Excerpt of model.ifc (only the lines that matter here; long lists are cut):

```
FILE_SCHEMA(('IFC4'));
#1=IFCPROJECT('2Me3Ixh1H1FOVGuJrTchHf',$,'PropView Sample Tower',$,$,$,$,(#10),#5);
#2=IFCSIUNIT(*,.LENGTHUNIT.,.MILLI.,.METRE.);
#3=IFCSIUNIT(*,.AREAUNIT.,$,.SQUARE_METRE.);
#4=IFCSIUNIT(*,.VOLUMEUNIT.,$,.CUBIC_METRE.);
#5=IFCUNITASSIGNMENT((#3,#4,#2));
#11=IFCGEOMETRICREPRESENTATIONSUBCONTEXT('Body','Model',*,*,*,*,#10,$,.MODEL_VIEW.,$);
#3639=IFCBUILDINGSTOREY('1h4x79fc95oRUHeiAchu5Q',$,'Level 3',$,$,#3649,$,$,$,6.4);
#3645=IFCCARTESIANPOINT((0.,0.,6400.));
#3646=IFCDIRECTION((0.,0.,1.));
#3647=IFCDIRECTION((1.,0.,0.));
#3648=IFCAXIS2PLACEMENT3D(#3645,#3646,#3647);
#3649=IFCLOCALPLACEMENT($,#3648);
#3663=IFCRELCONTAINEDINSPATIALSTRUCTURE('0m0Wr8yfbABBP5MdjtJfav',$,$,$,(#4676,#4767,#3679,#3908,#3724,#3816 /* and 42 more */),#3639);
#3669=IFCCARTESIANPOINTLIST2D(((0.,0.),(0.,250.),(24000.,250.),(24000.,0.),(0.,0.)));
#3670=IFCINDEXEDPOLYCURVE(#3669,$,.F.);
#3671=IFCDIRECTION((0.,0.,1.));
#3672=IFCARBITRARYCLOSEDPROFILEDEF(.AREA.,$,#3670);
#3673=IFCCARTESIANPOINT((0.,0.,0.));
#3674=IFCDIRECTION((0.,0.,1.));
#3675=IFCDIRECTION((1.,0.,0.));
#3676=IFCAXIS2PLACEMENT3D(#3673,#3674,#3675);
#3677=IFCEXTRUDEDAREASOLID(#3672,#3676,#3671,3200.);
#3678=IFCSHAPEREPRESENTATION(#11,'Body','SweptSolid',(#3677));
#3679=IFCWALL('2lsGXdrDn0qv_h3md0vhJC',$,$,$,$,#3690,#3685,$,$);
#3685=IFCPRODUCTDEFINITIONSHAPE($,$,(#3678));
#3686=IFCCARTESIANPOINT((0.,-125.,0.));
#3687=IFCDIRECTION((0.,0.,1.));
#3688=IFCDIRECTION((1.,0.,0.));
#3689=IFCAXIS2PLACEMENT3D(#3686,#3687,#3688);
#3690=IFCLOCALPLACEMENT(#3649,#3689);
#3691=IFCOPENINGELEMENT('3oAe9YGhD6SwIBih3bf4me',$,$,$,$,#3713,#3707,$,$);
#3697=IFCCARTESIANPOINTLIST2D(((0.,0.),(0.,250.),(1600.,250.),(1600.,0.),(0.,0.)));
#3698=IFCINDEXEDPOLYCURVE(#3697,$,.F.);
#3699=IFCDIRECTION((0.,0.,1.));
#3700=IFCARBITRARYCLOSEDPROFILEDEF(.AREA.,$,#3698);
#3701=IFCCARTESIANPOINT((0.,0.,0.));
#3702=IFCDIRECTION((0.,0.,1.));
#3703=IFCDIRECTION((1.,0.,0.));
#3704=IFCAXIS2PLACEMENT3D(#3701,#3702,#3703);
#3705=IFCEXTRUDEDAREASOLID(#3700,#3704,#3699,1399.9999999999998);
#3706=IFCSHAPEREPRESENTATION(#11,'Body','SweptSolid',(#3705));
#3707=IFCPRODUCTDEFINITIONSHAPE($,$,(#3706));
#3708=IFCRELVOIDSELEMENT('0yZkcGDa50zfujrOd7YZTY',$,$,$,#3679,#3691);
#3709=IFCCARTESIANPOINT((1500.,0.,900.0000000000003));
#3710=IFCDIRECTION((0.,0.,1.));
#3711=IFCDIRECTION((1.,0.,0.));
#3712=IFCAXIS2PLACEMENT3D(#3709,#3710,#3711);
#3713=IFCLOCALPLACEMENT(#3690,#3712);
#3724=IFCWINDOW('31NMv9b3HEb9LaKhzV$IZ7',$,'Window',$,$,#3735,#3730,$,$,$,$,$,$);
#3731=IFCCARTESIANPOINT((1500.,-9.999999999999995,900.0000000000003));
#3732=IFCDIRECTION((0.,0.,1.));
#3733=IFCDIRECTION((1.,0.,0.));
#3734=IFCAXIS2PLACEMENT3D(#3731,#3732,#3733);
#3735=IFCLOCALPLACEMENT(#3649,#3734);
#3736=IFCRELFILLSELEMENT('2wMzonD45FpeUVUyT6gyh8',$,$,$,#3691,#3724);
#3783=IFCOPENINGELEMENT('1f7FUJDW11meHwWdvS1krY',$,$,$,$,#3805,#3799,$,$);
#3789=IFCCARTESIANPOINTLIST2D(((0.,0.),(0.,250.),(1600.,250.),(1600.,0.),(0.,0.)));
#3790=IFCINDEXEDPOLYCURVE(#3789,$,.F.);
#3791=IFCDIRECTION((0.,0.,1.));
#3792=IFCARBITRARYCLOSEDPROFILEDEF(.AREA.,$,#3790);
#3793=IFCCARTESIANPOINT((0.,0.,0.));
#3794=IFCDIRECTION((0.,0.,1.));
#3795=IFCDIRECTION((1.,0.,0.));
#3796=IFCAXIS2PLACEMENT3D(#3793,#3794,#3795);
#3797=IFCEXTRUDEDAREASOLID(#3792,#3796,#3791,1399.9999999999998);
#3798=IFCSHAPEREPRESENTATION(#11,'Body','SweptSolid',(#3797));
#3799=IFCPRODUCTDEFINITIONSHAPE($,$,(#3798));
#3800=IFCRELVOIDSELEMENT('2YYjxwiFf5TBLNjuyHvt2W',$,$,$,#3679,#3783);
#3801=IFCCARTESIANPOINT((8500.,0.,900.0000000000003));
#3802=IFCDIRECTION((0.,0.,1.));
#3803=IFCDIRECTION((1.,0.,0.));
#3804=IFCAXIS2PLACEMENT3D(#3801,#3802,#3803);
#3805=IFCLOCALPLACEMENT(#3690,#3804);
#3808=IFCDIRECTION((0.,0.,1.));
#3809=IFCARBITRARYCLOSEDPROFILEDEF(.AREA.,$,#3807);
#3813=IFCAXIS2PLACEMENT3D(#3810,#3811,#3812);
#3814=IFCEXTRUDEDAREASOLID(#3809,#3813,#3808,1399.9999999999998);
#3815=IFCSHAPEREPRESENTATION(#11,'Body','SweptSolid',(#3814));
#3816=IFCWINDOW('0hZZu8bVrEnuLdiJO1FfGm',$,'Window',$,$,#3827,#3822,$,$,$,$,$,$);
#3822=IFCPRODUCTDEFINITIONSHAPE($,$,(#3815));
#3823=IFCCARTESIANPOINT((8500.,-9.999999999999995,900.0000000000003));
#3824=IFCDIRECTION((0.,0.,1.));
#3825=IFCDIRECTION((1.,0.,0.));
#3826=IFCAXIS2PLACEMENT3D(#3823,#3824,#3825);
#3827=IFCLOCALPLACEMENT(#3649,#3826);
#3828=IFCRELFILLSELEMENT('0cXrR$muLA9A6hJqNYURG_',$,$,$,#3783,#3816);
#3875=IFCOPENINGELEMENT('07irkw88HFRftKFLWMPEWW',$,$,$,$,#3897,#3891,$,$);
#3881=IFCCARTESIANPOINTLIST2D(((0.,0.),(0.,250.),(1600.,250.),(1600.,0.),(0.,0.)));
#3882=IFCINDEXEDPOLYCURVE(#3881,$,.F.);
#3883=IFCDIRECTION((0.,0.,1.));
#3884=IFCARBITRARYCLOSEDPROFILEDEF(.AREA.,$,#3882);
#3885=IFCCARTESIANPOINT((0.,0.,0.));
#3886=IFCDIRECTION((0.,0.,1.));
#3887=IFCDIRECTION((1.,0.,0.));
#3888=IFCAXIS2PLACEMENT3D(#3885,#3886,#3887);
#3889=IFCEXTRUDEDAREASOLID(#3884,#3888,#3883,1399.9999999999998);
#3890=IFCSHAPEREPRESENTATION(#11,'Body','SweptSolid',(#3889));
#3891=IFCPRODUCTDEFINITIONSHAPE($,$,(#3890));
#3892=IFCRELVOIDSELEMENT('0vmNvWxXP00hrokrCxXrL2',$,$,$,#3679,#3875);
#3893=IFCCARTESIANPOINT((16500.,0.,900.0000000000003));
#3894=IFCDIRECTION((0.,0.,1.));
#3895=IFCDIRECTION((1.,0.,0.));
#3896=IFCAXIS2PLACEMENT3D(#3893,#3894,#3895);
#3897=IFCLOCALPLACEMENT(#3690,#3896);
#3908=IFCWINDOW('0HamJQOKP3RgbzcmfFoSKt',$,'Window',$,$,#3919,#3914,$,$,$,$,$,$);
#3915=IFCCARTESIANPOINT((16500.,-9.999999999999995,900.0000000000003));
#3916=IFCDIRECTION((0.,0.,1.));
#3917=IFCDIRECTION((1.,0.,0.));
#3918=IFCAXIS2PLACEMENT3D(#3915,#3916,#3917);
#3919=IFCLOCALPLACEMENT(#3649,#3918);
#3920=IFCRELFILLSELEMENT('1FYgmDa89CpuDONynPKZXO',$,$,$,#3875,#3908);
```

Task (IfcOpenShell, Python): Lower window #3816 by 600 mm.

```python
import numpy as np
import ifcopenshell
import ifcopenshell.api.geometry
import ifcopenshell.util.placement
import ifcopenshell.util.unit

model = ifcopenshell.open("model.ifc")
unit_scale = ifcopenshell.util.unit.calculate_unit_scale(model)

window = model.by_guid("0hZZu8bVrEnuLdiJO1FfGm")
opening = window.FillsVoids[0].RelatingOpeningElement
dz = -600.0

shift = np.array([0.0, 0.0, dz])
# The window is not placed relative to its opening, so move both.
for product in (opening, window):
    matrix = ifcopenshell.util.placement.get_local_placement(product.ObjectPlacement)
    matrix[:3, 3] += shift
    ifcopenshell.api.geometry.edit_object_placement(model, product=product, matrix=matrix, is_si=False)

print(f"moved by {dz * unit_scale:+.3f} m")

model.write("model_rev.ifc")
```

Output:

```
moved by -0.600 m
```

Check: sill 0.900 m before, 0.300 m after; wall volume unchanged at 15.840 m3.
